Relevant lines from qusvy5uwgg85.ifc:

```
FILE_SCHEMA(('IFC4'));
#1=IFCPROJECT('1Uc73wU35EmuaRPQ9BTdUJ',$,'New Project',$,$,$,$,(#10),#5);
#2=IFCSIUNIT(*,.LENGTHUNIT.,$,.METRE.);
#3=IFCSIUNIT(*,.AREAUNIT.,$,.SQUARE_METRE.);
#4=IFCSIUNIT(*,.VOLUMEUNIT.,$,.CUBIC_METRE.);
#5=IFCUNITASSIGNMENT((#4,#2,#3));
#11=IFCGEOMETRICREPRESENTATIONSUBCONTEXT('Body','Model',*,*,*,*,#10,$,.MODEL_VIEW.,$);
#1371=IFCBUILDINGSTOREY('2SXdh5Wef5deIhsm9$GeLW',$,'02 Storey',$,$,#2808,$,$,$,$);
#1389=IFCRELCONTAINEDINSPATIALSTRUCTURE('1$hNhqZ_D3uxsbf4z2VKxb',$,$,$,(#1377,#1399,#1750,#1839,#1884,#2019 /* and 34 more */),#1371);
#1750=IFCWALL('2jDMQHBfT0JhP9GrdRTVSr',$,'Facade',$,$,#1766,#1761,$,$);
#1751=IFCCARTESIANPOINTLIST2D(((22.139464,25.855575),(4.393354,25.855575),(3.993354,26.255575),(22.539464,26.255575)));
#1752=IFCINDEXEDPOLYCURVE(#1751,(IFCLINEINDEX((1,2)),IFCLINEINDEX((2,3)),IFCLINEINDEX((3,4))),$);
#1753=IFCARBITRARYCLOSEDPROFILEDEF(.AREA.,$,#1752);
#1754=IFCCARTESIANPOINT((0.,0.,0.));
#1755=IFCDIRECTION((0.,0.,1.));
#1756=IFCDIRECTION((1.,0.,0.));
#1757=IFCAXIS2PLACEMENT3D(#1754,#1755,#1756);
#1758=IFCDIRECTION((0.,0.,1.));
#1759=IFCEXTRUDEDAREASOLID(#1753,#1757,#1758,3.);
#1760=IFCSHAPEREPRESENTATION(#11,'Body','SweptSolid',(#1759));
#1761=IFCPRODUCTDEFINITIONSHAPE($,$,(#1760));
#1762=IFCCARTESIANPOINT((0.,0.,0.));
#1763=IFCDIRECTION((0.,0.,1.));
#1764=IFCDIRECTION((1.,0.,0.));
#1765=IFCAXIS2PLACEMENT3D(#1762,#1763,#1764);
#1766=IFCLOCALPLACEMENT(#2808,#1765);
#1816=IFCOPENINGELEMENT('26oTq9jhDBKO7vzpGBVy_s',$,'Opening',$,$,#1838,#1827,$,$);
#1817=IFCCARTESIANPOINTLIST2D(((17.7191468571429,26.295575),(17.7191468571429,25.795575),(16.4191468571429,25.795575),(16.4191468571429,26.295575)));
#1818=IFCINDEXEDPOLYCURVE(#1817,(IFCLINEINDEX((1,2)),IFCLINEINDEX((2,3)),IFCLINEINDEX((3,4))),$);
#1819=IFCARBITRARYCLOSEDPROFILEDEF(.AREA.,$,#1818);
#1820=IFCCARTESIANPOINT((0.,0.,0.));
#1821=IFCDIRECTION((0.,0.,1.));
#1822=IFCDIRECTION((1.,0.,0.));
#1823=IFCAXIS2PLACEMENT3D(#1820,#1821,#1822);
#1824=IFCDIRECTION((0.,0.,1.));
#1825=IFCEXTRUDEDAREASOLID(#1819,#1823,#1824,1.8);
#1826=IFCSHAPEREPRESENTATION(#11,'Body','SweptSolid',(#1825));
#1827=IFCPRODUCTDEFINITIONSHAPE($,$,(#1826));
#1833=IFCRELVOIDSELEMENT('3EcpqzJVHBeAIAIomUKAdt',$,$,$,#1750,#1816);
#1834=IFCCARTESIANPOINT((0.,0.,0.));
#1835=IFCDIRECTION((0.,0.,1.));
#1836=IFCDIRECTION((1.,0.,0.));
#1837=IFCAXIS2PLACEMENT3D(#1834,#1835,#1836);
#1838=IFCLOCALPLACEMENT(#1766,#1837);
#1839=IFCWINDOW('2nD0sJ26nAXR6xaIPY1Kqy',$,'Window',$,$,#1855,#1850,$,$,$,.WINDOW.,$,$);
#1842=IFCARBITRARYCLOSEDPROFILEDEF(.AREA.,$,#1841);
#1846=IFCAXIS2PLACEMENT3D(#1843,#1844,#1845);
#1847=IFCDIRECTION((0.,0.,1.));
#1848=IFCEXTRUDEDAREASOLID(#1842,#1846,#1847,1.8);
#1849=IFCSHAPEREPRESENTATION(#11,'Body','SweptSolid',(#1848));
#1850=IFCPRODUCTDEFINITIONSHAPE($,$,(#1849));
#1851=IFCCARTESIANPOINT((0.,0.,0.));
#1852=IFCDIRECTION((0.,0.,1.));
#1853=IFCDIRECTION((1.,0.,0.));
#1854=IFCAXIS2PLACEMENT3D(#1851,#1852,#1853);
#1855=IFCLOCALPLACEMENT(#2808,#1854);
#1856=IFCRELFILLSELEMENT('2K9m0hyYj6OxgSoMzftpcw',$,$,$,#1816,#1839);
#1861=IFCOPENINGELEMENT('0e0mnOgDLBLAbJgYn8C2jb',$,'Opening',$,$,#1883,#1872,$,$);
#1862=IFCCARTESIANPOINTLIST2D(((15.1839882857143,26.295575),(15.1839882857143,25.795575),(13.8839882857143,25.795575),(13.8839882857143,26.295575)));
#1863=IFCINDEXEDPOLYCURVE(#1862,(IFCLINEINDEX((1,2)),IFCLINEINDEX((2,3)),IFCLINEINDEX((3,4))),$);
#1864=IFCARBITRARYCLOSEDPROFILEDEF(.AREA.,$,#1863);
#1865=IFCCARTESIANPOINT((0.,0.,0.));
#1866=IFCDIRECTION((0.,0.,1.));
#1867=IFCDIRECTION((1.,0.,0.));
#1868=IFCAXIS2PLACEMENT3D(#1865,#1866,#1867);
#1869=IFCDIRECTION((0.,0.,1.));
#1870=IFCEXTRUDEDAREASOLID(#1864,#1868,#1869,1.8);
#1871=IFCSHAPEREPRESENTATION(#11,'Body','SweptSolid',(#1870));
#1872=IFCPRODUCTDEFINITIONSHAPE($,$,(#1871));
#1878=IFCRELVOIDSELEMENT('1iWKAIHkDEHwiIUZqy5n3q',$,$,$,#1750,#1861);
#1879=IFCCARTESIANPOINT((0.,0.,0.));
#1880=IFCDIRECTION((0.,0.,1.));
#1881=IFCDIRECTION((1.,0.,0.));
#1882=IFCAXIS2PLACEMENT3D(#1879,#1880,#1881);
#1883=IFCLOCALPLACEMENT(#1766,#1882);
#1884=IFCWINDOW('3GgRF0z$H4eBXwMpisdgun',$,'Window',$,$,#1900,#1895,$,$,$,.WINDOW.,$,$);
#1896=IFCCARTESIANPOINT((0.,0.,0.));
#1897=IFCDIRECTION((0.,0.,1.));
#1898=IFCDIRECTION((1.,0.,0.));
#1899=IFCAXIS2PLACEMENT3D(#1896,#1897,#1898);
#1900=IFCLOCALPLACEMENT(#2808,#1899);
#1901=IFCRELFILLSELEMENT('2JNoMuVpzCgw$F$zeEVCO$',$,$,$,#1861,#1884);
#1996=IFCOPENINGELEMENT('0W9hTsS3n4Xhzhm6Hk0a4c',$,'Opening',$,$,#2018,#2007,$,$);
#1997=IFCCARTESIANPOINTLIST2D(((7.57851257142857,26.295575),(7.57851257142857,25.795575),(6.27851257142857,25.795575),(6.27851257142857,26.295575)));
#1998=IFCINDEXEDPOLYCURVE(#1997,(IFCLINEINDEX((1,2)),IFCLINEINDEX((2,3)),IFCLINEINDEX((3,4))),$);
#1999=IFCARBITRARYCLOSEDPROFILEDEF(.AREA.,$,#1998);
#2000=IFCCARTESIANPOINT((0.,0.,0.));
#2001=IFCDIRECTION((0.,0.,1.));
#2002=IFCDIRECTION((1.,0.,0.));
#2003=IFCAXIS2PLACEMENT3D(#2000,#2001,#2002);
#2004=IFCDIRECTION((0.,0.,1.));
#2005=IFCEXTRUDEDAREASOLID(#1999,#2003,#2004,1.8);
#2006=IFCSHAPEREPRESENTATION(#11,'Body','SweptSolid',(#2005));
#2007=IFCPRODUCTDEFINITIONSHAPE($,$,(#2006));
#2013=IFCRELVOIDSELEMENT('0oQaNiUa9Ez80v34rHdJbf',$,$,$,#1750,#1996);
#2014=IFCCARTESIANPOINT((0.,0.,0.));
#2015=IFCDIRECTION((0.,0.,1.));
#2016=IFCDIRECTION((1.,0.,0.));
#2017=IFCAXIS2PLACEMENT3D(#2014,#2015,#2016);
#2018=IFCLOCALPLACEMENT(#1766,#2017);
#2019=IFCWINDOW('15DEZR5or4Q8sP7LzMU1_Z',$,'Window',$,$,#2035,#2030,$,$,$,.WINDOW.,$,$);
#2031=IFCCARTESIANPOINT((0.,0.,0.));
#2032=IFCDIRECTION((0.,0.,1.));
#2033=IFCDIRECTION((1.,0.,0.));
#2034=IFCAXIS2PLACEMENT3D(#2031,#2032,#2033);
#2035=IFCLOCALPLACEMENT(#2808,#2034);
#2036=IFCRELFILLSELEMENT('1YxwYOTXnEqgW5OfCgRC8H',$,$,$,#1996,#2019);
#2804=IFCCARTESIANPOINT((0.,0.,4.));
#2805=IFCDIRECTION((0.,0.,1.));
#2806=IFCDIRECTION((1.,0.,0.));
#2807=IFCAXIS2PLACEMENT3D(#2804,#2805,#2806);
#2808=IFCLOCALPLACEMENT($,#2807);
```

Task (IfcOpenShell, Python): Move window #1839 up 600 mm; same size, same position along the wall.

```python
import numpy as np
import ifcopenshell
import ifcopenshell.api.geometry
import ifcopenshell.util.placement
import ifcopenshell.util.unit

model = ifcopenshell.open("qusvy5uwgg85.ifc")
unit_scale = ifcopenshell.util.unit.calculate_unit_scale(model)

window = model.by_id(1839)
opening = window.FillsVoids[0].RelatingOpeningElement
dz = 0.6 / unit_scale

shift = np.array([0.0, 0.0, dz])
# The window is not placed relative to its opening, so move both.
for product in (opening, window):
    matrix = ifcopenshell.util.placement.get_local_placement(product.ObjectPlacement)
    matrix[:3, 3] += shift
    ifcopenshell.api.geometry.edit_object_placement(model, product=product, matrix=matrix, is_si=False)

print(f"moved by {dz * unit_scale:+.3f} m")

model.write("qusvy5uwgg85_edited.ifc")
```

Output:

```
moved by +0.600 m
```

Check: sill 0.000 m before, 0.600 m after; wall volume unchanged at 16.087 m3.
